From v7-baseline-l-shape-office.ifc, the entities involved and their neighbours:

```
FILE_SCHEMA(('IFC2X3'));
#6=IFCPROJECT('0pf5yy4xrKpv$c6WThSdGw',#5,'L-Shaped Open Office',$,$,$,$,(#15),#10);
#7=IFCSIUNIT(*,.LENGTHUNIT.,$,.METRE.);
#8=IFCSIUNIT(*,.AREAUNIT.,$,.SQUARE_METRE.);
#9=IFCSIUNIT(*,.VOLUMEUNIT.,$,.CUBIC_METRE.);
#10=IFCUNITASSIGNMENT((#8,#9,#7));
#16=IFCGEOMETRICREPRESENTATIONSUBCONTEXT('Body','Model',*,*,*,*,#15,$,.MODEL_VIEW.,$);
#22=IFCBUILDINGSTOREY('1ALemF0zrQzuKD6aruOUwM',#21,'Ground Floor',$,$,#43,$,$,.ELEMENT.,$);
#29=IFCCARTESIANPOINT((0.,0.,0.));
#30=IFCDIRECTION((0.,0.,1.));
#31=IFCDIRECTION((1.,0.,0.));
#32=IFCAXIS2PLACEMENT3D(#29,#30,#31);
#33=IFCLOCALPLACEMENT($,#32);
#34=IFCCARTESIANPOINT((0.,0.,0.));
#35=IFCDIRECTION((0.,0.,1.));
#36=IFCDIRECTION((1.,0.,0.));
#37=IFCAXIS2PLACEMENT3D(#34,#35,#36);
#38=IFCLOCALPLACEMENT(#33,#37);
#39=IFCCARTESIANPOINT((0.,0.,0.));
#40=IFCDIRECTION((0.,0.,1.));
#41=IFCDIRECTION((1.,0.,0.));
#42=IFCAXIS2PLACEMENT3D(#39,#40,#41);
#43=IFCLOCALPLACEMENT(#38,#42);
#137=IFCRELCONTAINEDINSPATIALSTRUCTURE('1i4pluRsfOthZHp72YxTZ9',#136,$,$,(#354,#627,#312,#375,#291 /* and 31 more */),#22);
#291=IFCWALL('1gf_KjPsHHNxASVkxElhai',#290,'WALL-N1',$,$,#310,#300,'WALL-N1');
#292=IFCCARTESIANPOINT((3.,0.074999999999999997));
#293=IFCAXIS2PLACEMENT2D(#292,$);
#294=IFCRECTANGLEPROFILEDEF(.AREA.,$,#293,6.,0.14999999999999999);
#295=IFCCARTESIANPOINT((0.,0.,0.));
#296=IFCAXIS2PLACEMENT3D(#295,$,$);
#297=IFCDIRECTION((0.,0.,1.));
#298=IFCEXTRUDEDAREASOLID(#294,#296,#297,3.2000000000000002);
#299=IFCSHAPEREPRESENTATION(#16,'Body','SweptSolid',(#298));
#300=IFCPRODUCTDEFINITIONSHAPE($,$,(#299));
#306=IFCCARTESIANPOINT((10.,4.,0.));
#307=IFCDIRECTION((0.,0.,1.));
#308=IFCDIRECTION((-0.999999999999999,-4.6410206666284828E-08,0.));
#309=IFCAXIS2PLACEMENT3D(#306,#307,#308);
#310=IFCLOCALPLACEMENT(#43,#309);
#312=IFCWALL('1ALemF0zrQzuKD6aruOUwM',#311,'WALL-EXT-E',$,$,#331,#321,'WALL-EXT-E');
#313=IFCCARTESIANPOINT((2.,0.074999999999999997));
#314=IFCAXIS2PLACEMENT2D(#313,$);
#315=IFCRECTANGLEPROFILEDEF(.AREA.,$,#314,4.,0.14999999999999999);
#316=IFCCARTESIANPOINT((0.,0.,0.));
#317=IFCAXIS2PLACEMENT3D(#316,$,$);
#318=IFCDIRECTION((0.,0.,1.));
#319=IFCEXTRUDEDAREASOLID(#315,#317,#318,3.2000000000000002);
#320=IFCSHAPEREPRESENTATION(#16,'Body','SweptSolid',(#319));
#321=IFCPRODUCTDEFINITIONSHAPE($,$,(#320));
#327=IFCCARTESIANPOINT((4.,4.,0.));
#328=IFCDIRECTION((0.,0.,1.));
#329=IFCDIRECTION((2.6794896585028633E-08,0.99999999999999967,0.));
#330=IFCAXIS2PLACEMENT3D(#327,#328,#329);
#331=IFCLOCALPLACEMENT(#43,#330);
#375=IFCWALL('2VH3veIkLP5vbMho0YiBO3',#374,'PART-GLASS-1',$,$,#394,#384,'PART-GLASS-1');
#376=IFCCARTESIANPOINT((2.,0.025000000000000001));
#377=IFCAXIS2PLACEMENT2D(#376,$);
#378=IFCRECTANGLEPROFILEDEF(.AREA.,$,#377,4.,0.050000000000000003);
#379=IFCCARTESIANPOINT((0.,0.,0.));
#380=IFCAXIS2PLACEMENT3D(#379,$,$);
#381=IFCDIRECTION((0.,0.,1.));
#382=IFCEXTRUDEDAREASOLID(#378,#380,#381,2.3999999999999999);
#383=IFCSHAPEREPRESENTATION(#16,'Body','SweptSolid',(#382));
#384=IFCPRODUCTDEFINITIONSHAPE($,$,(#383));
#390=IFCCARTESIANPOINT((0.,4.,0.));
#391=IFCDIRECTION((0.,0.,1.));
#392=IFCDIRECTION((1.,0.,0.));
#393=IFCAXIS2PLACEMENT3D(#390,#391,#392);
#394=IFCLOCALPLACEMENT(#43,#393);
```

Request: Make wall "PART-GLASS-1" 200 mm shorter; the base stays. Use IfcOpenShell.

```python
import ifcopenshell
import ifcopenshell.geom
import ifcopenshell.util.representation
import ifcopenshell.util.shape

model = ifcopenshell.open("v7-baseline-l-shape-office.ifc")
settings = ifcopenshell.geom.settings()


def volume(element):
    """Net volume in cubic metres, openings subtracted."""
    shape = ifcopenshell.geom.create_shape(settings, element)
    return ifcopenshell.util.shape.get_volume(shape.geometry)


wall = model.by_id(375)
before = volume(wall)

body = ifcopenshell.util.representation.get_representation(wall, "Model", "Body")
solid = body.Items[0]
old_height = solid.Depth
solid.Depth -= 0.2
after = volume(wall)

print(f"height {old_height:g} -> {solid.Depth:g}, volume {before:.3f} -> {after:.3f} m3")

model.write("v7-baseline-l-shape-office_updated.ifc")
```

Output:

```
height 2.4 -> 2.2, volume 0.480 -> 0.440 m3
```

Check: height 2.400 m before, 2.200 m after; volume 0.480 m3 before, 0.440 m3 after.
